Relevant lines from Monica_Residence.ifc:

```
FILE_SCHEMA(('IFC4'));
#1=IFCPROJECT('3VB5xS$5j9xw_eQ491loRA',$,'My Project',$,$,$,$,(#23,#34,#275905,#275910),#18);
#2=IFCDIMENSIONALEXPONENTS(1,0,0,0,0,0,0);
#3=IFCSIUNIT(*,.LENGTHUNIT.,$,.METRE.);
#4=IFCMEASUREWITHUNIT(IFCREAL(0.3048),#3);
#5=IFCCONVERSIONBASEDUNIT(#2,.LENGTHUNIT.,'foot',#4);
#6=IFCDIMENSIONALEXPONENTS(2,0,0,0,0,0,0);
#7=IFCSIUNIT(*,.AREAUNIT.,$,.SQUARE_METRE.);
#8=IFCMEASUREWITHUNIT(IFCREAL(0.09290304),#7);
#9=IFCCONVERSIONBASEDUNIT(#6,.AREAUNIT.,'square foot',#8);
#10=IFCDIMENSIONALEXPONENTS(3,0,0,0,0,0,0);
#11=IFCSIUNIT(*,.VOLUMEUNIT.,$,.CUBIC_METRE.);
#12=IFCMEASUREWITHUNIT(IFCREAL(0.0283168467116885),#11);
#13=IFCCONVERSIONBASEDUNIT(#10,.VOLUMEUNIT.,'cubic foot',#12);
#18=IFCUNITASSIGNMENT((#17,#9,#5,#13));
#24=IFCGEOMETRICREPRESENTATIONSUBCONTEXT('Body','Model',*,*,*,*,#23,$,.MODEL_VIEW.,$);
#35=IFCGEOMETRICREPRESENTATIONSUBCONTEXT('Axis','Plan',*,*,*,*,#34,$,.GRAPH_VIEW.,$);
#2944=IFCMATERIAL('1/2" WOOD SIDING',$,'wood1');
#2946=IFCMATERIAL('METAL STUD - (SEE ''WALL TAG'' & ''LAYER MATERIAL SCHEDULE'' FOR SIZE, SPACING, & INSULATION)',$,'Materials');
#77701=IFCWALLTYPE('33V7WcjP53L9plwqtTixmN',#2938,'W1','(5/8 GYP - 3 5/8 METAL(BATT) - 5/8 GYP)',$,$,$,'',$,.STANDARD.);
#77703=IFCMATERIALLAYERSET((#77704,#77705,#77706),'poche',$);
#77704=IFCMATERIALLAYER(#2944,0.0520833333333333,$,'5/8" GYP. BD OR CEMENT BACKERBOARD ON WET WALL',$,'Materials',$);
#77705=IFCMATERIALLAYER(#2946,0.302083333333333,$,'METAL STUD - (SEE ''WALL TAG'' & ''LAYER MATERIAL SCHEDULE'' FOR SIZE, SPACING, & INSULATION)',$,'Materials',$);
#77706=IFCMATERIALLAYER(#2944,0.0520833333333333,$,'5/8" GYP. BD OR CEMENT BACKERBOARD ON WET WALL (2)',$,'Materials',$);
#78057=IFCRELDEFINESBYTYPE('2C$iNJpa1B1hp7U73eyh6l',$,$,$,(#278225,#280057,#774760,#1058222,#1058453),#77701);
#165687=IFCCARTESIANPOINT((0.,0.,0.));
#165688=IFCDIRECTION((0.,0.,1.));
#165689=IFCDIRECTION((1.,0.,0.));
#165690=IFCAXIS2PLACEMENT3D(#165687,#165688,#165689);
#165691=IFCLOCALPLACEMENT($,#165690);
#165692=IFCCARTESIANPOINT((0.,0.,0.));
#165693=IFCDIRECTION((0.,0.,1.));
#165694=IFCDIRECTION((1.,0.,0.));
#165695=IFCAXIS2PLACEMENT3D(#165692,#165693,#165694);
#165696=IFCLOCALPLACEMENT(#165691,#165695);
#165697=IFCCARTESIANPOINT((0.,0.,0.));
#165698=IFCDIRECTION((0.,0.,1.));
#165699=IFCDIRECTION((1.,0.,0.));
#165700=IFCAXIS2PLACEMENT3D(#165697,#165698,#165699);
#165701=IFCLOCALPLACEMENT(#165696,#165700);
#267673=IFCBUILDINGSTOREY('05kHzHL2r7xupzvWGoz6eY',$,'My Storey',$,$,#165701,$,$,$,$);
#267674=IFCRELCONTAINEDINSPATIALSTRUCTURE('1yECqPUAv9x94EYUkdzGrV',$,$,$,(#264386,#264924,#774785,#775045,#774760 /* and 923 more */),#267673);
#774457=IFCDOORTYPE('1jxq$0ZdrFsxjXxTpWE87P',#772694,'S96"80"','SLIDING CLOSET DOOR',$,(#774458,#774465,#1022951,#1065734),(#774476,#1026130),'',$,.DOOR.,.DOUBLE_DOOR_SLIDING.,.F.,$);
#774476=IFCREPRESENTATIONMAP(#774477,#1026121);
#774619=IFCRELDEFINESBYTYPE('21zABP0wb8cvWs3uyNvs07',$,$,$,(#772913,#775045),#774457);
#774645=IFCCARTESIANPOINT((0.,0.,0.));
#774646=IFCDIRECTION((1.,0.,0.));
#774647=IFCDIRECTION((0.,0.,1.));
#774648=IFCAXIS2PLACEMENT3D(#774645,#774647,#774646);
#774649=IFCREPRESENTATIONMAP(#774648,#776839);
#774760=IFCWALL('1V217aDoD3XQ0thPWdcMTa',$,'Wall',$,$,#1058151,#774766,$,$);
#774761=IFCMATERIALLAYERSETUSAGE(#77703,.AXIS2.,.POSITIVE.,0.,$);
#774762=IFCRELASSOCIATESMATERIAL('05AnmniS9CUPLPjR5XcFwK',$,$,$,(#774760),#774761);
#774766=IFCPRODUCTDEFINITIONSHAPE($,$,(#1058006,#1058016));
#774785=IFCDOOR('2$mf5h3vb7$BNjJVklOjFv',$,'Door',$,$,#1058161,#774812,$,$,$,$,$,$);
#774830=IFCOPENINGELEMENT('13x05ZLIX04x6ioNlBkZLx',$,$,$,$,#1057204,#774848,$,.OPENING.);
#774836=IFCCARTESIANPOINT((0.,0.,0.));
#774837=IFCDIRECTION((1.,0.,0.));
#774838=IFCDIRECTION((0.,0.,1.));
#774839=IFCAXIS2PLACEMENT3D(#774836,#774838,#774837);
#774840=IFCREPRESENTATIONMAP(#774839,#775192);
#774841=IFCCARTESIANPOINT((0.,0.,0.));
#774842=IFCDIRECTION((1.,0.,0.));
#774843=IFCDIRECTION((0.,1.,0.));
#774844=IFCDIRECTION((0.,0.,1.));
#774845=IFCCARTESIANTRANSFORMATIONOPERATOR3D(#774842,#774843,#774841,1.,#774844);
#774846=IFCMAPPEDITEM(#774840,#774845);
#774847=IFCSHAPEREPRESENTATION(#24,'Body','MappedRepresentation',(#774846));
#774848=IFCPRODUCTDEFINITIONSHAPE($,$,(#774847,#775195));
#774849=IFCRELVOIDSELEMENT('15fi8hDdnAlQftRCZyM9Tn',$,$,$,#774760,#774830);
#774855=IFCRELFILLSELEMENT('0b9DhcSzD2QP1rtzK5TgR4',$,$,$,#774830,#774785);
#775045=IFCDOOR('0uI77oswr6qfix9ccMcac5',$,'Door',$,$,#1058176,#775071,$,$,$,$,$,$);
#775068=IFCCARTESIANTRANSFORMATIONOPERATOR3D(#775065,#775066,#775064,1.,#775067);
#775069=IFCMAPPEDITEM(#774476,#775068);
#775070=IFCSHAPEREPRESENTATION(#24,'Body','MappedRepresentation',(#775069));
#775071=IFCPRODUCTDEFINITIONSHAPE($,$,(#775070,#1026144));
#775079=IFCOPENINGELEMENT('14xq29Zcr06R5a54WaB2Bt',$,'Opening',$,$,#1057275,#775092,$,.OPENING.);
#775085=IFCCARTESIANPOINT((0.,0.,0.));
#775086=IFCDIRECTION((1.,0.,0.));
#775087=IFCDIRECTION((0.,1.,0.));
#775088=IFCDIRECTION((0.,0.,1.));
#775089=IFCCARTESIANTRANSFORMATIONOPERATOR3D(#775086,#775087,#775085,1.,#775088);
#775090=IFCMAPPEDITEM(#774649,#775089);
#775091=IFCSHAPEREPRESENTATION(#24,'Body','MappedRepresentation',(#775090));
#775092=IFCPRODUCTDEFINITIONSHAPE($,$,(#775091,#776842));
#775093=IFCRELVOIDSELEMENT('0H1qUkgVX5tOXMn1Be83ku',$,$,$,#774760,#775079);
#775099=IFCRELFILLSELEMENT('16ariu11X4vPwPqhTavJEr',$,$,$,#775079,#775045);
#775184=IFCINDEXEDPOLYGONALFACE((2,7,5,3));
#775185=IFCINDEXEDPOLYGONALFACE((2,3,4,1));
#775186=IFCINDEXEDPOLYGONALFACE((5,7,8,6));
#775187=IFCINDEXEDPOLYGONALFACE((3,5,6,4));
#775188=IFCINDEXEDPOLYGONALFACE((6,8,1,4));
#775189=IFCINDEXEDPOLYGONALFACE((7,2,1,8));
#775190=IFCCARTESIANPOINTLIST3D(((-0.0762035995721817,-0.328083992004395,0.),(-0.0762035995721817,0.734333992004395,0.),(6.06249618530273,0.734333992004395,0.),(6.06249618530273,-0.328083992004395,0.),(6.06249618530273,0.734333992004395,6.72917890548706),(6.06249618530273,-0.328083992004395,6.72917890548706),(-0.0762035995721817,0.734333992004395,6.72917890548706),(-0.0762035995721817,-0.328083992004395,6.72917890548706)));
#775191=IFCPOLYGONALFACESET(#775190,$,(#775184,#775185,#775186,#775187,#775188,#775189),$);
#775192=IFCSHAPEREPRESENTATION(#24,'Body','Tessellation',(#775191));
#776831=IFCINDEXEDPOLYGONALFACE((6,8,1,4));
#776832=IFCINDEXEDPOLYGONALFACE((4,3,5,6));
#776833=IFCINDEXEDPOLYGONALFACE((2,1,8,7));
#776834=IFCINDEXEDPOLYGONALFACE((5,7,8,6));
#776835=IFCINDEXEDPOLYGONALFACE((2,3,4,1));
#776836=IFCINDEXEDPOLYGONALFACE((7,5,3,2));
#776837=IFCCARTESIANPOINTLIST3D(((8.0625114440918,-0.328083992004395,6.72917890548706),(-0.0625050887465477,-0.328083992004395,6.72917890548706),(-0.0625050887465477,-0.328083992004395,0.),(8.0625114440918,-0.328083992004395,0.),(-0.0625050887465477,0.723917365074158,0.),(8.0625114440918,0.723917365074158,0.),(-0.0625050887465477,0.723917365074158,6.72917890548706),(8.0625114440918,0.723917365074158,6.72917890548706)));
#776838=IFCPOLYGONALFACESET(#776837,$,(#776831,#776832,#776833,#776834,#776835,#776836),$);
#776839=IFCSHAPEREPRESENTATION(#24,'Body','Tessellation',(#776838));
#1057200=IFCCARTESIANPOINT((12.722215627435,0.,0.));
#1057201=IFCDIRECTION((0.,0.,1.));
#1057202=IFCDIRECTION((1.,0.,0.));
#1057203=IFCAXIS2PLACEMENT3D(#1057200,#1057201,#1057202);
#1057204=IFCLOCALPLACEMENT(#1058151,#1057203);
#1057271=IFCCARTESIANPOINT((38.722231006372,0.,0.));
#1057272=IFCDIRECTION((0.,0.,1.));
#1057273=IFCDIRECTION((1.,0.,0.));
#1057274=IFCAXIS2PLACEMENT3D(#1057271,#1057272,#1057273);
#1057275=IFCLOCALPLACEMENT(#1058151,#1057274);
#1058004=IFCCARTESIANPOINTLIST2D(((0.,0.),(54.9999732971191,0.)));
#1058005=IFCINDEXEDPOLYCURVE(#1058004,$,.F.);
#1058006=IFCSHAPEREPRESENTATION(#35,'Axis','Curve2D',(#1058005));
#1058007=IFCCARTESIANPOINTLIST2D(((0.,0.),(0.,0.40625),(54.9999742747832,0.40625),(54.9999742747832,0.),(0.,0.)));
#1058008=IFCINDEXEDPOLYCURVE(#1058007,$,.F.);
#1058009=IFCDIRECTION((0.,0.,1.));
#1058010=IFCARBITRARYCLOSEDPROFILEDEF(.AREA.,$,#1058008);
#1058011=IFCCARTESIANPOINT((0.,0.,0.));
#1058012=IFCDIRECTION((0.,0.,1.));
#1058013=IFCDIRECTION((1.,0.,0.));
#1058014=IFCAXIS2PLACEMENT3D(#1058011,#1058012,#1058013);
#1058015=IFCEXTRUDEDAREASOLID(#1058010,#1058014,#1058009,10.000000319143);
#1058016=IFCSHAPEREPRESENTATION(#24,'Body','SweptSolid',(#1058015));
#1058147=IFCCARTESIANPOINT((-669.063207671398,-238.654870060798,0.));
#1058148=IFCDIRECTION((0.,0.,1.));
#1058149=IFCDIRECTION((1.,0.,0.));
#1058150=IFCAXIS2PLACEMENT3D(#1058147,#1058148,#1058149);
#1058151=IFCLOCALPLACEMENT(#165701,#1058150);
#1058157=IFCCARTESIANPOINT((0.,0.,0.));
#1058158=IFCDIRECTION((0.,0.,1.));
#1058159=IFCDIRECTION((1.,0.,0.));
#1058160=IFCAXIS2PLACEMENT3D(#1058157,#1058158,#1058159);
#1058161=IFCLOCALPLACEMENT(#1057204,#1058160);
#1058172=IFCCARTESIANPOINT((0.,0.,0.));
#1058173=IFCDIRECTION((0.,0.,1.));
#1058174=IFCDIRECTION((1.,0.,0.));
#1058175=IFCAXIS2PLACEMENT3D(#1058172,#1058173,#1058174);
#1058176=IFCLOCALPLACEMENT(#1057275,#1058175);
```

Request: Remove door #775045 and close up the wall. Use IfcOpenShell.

```python
import ifcopenshell
import ifcopenshell.api.feature
import ifcopenshell.api.root
import ifcopenshell.geom
import ifcopenshell.util.shape

model = ifcopenshell.open("Monica_Residence.ifc")
settings = ifcopenshell.geom.settings()


def volume(element):
    """Net volume in cubic metres, openings subtracted."""
    shape = ifcopenshell.geom.create_shape(settings, element)
    return ifcopenshell.util.shape.get_volume(shape.geometry)


door = model.by_guid("0uI77oswr6qfix9ccMcac5")
opening = door.FillsVoids[0].RelatingOpeningElement
wall = opening.VoidsElements[0].RelatingBuildingElement
before = volume(wall)

ifcopenshell.api.root.remove_product(model, product=door)
ifcopenshell.api.feature.remove_feature(model, feature=opening)

after = volume(wall)

print(f"wall volume {before:.3f} -> {after:.3f} m3")

model.write("Monica_Residence_updated.ifc")
```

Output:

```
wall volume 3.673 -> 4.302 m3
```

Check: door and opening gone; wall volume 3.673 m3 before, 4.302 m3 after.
